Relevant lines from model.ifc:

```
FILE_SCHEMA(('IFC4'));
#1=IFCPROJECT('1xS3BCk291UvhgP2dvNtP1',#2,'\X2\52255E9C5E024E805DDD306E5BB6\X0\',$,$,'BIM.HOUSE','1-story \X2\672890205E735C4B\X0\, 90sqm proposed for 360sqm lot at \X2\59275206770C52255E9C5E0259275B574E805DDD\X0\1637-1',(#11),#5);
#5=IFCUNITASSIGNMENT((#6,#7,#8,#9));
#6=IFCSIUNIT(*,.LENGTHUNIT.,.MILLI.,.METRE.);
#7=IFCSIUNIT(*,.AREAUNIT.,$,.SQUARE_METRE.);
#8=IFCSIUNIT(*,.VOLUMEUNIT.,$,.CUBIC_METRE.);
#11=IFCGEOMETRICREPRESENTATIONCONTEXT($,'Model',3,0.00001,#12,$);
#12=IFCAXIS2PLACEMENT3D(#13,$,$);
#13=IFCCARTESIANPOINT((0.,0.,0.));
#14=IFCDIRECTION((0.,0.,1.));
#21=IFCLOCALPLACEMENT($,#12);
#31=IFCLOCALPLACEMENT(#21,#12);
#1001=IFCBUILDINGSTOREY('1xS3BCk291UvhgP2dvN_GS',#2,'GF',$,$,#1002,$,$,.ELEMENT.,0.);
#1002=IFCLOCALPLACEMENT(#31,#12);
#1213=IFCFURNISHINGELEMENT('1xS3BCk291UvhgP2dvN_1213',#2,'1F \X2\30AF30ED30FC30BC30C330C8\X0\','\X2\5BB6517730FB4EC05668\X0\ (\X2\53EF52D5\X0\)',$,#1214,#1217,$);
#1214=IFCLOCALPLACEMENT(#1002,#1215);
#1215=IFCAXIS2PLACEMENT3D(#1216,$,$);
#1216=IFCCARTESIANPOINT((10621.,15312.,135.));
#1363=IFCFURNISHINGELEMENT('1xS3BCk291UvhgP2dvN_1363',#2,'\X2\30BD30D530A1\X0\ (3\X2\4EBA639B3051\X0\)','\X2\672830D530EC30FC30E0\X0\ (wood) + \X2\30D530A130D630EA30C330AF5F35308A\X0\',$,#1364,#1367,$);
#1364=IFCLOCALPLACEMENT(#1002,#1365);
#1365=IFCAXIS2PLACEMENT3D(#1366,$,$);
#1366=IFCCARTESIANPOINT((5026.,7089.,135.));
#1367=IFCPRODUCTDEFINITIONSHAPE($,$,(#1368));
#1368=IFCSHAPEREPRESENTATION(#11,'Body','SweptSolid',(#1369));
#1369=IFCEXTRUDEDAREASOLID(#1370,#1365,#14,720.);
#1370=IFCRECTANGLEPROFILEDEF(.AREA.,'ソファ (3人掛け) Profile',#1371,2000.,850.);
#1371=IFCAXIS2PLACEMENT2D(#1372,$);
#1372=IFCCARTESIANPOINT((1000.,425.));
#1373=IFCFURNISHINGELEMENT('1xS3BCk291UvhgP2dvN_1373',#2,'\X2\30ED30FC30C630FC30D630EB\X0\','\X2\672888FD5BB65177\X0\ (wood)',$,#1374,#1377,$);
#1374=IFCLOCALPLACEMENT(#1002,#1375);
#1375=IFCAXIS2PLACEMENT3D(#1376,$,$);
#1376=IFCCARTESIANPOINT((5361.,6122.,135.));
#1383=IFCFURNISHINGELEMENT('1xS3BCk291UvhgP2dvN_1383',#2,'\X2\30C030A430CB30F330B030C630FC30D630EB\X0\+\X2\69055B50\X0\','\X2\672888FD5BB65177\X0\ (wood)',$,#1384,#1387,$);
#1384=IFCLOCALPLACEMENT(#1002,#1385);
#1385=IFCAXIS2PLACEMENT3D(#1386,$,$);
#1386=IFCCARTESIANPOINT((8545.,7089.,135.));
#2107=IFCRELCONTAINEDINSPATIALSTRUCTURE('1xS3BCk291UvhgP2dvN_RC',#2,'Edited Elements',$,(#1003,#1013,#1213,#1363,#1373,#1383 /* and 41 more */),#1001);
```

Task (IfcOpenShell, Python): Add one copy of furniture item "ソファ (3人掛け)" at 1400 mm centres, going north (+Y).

```python
import numpy as np
import ifcopenshell
import ifcopenshell.api.geometry
import ifcopenshell.api.root
import ifcopenshell.util.element
import ifcopenshell.util.placement
import ifcopenshell.util.unit

model = ifcopenshell.open("model.ifc")
unit_scale = ifcopenshell.util.unit.calculate_unit_scale(model)


def reuse_history(source, copy):
    """copy_class also copies each property set's owner history, people and application; keep the originals."""
    for rel in copy.IsDefinedBy:
        if rel.is_a("IfcRelDefinesByProperties") and (history := rel.RelatingPropertyDefinition.OwnerHistory):
            rel.RelatingPropertyDefinition.OwnerHistory = source.OwnerHistory
            ifcopenshell.util.element.remove_deep2(model, history)


source = model.by_guid("1xS3BCk291UvhgP2dvN_1363")
base = ifcopenshell.util.placement.get_local_placement(source.ObjectPlacement)
step = np.array([0.0, 1.0, 0.0]) * 1.4 / unit_scale

for i in range(1, 2):
    copy = ifcopenshell.api.root.copy_class(model, product=source)
    copy.Representation = ifcopenshell.util.element.copy_deep(
        model, source.Representation, exclude=["IfcGeometricRepresentationContext", "IfcRepresentationMap"]
    )
    reuse_history(source, copy)
    matrix = base.copy()
    matrix[:3, 3] += i * step
    print("added at", matrix[:3, 3].round(3) + 0.0)
    ifcopenshell.api.geometry.edit_object_placement(model, product=copy, matrix=matrix, is_si=False)

model.write("model_edited.ifc")
```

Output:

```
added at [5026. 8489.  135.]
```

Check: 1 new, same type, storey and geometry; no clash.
